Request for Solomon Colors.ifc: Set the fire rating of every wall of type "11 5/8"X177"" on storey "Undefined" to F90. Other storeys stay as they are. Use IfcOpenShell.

First a look at what the model holds.

```python
import ifcopenshell
import ifcopenshell.util.element

model = ifcopenshell.open("Solomon Colors.ifc")
print(model.schema)
storey = next(s for s in model.by_type("IfcBuildingStorey") if s.Name == "Undefined")
walls = [e for e in ifcopenshell.util.element.get_decomposition(storey) if e.is_a("IfcWall")]
seen = {}
for e in walls:
    element_type = ifcopenshell.util.element.get_type(e)
    key = (element_type.Name if element_type != e and element_type else None, ifcopenshell.util.element.get_pset(e, "Pset_WallCommon", "FireRating"))
    seen[key] = seen.get(key, 0) + 1
for (name, value), count in sorted(seen.items(), key=str):
    print(count, "x", name, "|", value)
```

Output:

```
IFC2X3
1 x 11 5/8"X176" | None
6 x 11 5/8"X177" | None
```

```python
import ifcopenshell
import ifcopenshell.api.pset
import ifcopenshell.util.element

model = ifcopenshell.open("Solomon Colors.ifc")

storey = next(s for s in model.by_type("IfcBuildingStorey") if s.Name == "Undefined")
walls = [e for e in ifcopenshell.util.element.get_decomposition(storey) if e.is_a("IfcWall")]

count = 0
for e in walls:
    element_type = ifcopenshell.util.element.get_type(e)
    if element_type in (None, e) or element_type.Name != '11 5/8"X177"':
        continue
    # add_pset returns the element's existing set when there is one.
    pset = ifcopenshell.api.pset.add_pset(model, product=e, name="Pset_WallCommon")
    ifcopenshell.api.pset.edit_pset(model, pset=pset, properties={"FireRating": "F90"})
    count += 1

print(count, "walls updated")

model.write("Solomon Colors_v2.ifc")
```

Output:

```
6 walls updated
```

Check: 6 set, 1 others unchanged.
